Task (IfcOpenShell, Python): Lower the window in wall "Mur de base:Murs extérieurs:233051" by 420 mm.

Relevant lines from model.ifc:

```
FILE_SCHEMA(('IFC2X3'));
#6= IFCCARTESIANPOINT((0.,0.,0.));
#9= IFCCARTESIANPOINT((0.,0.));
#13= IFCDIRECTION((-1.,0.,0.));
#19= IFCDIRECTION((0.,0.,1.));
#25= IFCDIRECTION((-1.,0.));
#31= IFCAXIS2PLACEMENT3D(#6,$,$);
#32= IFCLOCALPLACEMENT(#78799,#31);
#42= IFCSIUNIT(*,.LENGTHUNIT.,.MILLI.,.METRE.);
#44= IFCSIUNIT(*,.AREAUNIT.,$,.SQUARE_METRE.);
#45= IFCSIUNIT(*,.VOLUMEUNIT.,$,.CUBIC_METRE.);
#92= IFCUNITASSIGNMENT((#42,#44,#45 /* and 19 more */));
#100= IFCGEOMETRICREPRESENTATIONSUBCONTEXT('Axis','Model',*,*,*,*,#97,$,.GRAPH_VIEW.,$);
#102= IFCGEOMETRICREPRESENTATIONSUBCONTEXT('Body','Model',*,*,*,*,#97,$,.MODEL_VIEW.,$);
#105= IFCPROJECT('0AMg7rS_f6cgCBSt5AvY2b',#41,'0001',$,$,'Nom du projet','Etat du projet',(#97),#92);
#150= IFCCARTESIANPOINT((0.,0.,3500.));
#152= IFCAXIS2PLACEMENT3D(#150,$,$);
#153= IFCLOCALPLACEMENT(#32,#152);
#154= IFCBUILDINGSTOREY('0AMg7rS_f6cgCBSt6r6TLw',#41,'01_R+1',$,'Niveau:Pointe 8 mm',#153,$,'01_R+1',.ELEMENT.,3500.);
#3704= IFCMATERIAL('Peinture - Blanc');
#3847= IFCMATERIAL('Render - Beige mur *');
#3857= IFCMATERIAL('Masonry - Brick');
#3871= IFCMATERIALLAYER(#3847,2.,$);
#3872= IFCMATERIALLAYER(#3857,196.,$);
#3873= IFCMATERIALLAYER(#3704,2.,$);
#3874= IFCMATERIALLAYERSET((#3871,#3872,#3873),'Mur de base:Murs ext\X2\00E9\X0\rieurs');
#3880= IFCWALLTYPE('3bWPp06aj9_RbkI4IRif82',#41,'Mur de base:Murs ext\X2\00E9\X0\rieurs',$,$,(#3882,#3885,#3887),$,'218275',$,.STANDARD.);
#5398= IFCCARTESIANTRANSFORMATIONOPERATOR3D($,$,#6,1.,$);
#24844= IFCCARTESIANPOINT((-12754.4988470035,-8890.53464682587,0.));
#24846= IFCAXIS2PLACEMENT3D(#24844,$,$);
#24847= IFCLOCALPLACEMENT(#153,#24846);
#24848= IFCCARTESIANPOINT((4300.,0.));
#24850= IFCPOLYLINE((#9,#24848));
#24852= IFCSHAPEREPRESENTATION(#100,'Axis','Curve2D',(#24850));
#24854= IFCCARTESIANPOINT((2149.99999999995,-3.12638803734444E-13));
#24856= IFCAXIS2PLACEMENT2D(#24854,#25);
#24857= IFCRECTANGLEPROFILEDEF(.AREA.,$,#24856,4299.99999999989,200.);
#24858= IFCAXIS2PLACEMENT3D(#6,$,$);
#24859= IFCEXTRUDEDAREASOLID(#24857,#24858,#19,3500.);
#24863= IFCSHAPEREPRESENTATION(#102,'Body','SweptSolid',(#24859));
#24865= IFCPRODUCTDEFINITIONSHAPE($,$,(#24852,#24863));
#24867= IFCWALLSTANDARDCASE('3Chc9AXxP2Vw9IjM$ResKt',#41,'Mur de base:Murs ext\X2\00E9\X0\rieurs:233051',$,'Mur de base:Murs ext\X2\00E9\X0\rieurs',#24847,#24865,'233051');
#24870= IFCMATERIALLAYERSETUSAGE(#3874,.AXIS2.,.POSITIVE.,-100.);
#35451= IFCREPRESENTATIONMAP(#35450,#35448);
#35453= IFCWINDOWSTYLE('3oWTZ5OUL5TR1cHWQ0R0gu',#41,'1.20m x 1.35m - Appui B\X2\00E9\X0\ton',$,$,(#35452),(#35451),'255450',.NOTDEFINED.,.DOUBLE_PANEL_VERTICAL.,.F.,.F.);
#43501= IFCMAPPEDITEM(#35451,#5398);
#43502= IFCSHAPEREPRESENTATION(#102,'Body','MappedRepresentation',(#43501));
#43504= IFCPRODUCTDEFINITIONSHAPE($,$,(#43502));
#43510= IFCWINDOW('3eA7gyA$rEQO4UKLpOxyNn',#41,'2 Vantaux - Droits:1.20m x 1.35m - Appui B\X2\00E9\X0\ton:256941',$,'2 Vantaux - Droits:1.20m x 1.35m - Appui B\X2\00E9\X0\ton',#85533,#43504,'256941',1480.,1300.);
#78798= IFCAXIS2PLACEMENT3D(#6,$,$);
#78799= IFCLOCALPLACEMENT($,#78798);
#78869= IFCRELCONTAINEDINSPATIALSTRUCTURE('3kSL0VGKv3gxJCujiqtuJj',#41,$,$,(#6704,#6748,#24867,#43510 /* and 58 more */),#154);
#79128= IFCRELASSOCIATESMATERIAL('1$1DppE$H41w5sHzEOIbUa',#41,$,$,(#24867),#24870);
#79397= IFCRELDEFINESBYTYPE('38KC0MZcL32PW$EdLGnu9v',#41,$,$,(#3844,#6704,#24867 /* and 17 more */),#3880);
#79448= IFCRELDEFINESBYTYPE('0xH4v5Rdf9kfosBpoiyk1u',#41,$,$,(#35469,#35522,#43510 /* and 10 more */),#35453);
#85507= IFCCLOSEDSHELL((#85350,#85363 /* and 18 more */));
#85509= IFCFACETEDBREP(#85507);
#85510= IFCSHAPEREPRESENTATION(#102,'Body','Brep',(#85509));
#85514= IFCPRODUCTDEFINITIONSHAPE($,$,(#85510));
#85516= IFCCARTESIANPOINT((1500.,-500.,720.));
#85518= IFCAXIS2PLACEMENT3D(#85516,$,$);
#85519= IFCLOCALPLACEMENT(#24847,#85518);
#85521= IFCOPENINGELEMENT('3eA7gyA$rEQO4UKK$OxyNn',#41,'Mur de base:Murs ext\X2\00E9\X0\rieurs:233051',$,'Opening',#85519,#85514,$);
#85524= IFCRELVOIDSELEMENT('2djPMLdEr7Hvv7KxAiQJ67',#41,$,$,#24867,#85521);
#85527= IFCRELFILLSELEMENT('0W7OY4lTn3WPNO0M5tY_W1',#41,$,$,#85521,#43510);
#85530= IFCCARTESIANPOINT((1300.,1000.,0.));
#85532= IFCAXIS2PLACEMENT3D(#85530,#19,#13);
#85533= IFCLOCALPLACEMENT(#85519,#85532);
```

```python
import numpy as np
import ifcopenshell
import ifcopenshell.api.geometry
import ifcopenshell.util.placement
import ifcopenshell.util.unit

model = ifcopenshell.open("model.ifc")
unit_scale = ifcopenshell.util.unit.calculate_unit_scale(model)

window = model.by_id(43510)
opening = window.FillsVoids[0].RelatingOpeningElement
dz = -0.42 / unit_scale

shift = np.array([0.0, 0.0, dz])
# The window is placed relative to its opening, so it follows when the opening moves.
matrix = ifcopenshell.util.placement.get_local_placement(opening.ObjectPlacement)
matrix[:3, 3] += shift
ifcopenshell.api.geometry.edit_object_placement(
    model, product=opening, matrix=matrix, is_si=False, should_transform_children=True
)

print(f"moved by {dz * unit_scale:+.3f} m")

model.write("model_edited.ifc")
```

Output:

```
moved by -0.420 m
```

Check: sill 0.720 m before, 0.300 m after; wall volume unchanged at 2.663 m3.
